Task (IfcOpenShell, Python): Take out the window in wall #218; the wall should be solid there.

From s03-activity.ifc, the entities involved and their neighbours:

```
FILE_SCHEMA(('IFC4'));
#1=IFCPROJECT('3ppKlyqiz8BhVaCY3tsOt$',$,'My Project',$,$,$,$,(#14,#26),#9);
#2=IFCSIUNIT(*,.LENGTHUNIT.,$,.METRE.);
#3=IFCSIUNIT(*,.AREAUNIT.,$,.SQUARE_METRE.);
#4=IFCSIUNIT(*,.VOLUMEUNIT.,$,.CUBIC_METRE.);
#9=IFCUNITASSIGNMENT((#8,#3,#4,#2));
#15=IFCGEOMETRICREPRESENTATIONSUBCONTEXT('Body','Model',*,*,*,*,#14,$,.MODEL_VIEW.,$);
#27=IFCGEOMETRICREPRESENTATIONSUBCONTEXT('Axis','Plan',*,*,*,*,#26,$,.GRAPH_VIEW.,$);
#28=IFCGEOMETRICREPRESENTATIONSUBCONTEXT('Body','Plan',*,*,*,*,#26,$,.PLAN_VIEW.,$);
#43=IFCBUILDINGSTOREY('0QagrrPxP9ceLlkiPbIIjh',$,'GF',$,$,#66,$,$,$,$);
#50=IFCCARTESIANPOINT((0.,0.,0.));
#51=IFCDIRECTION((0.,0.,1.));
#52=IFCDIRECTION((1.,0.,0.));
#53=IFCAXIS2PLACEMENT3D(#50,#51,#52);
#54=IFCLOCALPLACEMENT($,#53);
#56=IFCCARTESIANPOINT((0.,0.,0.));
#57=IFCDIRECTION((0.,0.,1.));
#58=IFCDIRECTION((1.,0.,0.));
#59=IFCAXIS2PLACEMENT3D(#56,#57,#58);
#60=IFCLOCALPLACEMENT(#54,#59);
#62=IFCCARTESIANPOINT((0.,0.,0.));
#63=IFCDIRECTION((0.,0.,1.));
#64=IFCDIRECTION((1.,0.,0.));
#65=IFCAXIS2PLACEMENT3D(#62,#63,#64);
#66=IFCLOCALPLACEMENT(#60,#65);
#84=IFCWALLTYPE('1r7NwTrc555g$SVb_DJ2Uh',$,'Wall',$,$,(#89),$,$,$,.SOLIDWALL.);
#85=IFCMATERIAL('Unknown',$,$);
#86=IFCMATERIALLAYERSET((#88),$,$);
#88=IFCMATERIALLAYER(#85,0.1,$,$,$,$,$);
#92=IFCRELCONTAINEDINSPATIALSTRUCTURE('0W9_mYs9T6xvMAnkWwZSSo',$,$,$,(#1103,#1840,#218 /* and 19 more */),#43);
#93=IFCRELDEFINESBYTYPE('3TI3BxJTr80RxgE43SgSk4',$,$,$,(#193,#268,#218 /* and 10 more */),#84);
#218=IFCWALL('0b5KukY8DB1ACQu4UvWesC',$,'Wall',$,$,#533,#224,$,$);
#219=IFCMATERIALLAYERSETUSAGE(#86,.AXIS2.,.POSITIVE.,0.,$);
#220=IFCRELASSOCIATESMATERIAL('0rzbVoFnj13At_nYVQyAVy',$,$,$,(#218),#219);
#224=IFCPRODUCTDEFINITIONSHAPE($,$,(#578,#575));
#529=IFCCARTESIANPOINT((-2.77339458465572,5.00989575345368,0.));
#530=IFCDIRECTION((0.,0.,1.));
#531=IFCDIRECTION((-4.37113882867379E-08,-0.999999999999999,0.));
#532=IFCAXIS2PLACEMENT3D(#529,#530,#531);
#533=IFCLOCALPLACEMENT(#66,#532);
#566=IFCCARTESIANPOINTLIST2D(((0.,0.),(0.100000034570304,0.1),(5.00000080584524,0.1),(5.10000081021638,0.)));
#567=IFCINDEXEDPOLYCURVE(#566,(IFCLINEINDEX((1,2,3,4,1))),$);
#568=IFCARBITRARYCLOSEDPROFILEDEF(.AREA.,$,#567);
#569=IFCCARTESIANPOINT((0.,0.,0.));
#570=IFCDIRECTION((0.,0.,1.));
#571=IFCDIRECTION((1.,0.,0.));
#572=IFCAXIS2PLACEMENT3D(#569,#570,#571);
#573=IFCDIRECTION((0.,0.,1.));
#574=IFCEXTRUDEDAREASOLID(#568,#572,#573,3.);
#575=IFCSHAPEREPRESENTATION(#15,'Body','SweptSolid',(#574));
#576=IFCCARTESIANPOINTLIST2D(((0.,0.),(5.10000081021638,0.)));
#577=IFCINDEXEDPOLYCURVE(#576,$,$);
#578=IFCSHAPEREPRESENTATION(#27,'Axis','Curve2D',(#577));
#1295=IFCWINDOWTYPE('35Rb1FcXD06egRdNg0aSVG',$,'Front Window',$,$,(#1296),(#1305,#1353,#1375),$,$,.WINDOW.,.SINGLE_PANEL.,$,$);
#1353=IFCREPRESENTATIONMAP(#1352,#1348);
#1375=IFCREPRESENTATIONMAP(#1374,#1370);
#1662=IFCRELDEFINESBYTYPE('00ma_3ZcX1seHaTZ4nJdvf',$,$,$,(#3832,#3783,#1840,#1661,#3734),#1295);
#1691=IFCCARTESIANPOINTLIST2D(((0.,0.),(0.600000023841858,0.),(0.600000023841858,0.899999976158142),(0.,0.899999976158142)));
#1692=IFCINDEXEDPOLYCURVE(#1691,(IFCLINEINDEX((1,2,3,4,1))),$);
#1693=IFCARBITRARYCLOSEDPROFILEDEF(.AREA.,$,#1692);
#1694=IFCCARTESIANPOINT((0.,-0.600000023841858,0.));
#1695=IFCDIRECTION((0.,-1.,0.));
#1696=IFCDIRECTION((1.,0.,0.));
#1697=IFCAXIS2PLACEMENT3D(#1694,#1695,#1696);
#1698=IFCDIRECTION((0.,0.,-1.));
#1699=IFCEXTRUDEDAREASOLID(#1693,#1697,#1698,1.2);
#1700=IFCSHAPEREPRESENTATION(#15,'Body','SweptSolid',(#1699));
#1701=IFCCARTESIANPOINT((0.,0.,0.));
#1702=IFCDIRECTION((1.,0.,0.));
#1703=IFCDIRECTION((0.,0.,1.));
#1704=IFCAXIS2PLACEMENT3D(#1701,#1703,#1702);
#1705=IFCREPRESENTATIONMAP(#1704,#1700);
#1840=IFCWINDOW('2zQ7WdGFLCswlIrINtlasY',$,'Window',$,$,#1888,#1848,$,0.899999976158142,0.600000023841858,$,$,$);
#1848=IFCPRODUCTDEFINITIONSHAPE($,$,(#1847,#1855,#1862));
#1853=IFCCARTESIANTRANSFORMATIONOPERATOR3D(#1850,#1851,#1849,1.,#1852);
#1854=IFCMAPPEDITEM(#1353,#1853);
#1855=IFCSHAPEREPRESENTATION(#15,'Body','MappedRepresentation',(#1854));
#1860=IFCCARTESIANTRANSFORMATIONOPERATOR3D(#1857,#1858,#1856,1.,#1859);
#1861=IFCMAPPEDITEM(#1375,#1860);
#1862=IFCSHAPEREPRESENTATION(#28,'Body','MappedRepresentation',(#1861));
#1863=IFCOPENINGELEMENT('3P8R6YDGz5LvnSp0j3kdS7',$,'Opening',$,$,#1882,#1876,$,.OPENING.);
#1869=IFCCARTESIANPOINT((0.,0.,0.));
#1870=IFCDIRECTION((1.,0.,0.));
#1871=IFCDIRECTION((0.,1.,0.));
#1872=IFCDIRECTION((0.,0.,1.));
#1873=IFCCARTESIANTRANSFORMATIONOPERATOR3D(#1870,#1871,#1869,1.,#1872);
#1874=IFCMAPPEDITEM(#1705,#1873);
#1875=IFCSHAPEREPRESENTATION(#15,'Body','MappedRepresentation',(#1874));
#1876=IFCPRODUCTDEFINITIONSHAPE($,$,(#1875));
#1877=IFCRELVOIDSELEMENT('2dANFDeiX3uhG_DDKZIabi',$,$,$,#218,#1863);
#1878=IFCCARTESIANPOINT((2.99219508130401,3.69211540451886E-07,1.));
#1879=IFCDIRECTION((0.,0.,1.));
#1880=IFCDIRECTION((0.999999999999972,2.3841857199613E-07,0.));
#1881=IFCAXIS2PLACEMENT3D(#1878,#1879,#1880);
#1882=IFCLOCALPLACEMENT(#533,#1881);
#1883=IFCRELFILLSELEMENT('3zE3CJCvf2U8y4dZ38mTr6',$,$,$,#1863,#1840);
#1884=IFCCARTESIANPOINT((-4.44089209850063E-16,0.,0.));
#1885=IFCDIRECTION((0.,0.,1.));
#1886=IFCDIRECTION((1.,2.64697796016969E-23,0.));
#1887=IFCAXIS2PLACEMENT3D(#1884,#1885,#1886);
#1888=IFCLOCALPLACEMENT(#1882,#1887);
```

```python
import ifcopenshell
import ifcopenshell.api.feature
import ifcopenshell.api.root
import ifcopenshell.geom
import ifcopenshell.util.shape

model = ifcopenshell.open("s03-activity.ifc")
settings = ifcopenshell.geom.settings()


def volume(element):
    """Net volume in cubic metres, openings subtracted."""
    shape = ifcopenshell.geom.create_shape(settings, element)
    return ifcopenshell.util.shape.get_volume(shape.geometry)


window = model.by_guid("2zQ7WdGFLCswlIrINtlasY")
opening = window.FillsVoids[0].RelatingOpeningElement
wall = opening.VoidsElements[0].RelatingBuildingElement
before = volume(wall)

ifcopenshell.api.root.remove_product(model, product=window)
ifcopenshell.api.feature.remove_feature(model, feature=opening)

after = volume(wall)

print(f"wall volume {before:.3f} -> {after:.3f} m3")

model.write("s03-activity_v2.ifc")
```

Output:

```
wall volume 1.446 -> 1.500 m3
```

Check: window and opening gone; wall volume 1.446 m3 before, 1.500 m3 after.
